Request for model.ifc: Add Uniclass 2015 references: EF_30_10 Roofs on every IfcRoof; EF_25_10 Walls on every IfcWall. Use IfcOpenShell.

First a look at what the model holds.

```python
import ifcopenshell

model = ifcopenshell.open("model.ifc")
print(model.schema)
print("classifications:", [c.Name for c in model.by_type("IfcClassification")])
for ifc_class in ("IfcDoor", "IfcRoof", "IfcStair", "IfcWall", "IfcWindow"):
    print(ifc_class, len(model.by_type(ifc_class)))
```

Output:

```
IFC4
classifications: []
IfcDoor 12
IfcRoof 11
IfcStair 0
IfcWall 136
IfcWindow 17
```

```python
import ifcopenshell
import ifcopenshell.api.classification

model = ifcopenshell.open("model.ifc")

system = ifcopenshell.api.classification.add_classification(model, classification="Uniclass 2015")

codes = {
    "IfcRoof": ("EF_30_10", "Roofs"),
    "IfcWall": ("EF_25_10", "Walls"),
}
for ifc_class, (code, name) in codes.items():
    products = model.by_type(ifc_class)
    ifcopenshell.api.classification.add_reference(
        model, products=products, classification=system, identification=code, name=name
    )
    print(code, len(products))

model.write("model-out.ifc")
```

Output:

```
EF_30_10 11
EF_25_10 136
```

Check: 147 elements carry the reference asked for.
